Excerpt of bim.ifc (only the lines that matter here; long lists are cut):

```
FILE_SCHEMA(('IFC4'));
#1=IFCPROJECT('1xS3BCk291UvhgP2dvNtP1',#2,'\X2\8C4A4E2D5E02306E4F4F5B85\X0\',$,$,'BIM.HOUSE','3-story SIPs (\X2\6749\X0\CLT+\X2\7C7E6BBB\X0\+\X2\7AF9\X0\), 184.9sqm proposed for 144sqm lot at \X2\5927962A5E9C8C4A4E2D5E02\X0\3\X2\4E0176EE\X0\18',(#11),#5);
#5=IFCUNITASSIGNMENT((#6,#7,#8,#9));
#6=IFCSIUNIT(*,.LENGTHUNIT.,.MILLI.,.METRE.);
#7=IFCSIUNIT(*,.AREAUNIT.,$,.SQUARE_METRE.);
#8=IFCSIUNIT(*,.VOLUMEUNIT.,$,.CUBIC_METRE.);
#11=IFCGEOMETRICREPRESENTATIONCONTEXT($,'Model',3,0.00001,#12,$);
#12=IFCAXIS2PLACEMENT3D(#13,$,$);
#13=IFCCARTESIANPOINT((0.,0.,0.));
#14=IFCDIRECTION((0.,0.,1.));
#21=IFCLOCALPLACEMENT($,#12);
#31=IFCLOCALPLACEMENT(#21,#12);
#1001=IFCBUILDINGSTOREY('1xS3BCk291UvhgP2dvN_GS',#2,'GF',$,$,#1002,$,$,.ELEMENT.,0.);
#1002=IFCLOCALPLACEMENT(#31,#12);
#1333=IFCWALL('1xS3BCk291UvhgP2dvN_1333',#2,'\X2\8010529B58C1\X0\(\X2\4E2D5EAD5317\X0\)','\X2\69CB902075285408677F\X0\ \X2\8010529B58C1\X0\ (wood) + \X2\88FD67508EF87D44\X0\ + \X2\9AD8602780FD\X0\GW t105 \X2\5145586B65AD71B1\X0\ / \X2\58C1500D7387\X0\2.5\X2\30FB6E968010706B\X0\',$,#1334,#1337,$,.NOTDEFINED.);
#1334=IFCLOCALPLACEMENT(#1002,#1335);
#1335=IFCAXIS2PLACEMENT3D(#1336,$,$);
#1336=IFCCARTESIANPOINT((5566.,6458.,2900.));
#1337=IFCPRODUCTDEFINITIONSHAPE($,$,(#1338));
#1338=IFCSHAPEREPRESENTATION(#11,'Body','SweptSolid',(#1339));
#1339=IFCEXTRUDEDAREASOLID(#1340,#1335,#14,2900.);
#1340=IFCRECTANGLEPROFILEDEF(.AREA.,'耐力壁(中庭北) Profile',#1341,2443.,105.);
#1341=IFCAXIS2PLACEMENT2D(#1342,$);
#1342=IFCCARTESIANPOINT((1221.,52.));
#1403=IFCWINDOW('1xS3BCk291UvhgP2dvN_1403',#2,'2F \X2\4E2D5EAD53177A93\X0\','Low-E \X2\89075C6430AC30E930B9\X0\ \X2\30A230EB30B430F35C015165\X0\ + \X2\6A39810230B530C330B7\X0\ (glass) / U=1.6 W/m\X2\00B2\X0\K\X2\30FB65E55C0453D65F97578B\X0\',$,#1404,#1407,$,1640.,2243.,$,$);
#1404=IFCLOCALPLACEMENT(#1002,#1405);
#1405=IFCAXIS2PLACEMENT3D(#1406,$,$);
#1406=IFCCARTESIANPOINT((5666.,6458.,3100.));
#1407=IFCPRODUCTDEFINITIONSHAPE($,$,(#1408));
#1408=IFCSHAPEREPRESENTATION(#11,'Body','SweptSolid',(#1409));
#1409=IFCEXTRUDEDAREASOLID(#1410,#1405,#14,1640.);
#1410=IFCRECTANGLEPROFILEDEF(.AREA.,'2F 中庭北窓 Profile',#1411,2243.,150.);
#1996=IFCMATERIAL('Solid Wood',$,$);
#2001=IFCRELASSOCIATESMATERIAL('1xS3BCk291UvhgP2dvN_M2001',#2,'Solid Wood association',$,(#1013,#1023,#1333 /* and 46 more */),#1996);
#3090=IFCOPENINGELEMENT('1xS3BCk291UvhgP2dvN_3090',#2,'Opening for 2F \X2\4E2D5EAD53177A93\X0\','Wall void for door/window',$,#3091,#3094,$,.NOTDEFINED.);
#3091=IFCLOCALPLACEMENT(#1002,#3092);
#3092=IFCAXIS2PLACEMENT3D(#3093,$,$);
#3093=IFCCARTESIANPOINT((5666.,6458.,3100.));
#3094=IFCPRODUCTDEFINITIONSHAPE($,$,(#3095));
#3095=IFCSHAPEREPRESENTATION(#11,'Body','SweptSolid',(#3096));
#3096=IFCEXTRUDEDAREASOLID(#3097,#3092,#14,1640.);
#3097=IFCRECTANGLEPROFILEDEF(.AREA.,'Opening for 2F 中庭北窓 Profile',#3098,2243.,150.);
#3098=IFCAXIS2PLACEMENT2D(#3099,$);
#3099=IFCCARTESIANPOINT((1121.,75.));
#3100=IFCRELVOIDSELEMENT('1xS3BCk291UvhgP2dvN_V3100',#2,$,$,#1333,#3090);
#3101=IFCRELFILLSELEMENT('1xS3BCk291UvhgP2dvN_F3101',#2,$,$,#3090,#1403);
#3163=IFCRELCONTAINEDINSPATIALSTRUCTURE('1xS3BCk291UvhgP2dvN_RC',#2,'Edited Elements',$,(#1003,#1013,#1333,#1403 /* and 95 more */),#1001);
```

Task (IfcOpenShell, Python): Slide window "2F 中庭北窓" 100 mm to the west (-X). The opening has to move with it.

```python
import ifcopenshell
import ifcopenshell.api.geometry
import ifcopenshell.util.placement
import ifcopenshell.util.unit

model = ifcopenshell.open("bim.ifc")
unit_scale = ifcopenshell.util.unit.calculate_unit_scale(model)

window = model.by_guid("1xS3BCk291UvhgP2dvN_1403")
opening = window.FillsVoids[0].RelatingOpeningElement
wall = opening.VoidsElements[0].RelatingBuildingElement

wall_matrix = ifcopenshell.util.placement.get_local_placement(wall.ObjectPlacement)
shift = wall_matrix[:3, 0] * -0.1 / unit_scale
before = ifcopenshell.util.placement.get_local_placement(window.ObjectPlacement)[:3, 3].copy()

# The window is not placed relative to its opening, so move both.
for product in (opening, window):
    matrix = ifcopenshell.util.placement.get_local_placement(product.ObjectPlacement)
    matrix[:3, 3] += shift
    ifcopenshell.api.geometry.edit_object_placement(model, product=product, matrix=matrix, is_si=False)

after = ifcopenshell.util.placement.get_local_placement(window.ObjectPlacement)[:3, 3]
print("window moved by", (after - before).round(3) + 0.0)

model.write("bim_v2.ifc")
```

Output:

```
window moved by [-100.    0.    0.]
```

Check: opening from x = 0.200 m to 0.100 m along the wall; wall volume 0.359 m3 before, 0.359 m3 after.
